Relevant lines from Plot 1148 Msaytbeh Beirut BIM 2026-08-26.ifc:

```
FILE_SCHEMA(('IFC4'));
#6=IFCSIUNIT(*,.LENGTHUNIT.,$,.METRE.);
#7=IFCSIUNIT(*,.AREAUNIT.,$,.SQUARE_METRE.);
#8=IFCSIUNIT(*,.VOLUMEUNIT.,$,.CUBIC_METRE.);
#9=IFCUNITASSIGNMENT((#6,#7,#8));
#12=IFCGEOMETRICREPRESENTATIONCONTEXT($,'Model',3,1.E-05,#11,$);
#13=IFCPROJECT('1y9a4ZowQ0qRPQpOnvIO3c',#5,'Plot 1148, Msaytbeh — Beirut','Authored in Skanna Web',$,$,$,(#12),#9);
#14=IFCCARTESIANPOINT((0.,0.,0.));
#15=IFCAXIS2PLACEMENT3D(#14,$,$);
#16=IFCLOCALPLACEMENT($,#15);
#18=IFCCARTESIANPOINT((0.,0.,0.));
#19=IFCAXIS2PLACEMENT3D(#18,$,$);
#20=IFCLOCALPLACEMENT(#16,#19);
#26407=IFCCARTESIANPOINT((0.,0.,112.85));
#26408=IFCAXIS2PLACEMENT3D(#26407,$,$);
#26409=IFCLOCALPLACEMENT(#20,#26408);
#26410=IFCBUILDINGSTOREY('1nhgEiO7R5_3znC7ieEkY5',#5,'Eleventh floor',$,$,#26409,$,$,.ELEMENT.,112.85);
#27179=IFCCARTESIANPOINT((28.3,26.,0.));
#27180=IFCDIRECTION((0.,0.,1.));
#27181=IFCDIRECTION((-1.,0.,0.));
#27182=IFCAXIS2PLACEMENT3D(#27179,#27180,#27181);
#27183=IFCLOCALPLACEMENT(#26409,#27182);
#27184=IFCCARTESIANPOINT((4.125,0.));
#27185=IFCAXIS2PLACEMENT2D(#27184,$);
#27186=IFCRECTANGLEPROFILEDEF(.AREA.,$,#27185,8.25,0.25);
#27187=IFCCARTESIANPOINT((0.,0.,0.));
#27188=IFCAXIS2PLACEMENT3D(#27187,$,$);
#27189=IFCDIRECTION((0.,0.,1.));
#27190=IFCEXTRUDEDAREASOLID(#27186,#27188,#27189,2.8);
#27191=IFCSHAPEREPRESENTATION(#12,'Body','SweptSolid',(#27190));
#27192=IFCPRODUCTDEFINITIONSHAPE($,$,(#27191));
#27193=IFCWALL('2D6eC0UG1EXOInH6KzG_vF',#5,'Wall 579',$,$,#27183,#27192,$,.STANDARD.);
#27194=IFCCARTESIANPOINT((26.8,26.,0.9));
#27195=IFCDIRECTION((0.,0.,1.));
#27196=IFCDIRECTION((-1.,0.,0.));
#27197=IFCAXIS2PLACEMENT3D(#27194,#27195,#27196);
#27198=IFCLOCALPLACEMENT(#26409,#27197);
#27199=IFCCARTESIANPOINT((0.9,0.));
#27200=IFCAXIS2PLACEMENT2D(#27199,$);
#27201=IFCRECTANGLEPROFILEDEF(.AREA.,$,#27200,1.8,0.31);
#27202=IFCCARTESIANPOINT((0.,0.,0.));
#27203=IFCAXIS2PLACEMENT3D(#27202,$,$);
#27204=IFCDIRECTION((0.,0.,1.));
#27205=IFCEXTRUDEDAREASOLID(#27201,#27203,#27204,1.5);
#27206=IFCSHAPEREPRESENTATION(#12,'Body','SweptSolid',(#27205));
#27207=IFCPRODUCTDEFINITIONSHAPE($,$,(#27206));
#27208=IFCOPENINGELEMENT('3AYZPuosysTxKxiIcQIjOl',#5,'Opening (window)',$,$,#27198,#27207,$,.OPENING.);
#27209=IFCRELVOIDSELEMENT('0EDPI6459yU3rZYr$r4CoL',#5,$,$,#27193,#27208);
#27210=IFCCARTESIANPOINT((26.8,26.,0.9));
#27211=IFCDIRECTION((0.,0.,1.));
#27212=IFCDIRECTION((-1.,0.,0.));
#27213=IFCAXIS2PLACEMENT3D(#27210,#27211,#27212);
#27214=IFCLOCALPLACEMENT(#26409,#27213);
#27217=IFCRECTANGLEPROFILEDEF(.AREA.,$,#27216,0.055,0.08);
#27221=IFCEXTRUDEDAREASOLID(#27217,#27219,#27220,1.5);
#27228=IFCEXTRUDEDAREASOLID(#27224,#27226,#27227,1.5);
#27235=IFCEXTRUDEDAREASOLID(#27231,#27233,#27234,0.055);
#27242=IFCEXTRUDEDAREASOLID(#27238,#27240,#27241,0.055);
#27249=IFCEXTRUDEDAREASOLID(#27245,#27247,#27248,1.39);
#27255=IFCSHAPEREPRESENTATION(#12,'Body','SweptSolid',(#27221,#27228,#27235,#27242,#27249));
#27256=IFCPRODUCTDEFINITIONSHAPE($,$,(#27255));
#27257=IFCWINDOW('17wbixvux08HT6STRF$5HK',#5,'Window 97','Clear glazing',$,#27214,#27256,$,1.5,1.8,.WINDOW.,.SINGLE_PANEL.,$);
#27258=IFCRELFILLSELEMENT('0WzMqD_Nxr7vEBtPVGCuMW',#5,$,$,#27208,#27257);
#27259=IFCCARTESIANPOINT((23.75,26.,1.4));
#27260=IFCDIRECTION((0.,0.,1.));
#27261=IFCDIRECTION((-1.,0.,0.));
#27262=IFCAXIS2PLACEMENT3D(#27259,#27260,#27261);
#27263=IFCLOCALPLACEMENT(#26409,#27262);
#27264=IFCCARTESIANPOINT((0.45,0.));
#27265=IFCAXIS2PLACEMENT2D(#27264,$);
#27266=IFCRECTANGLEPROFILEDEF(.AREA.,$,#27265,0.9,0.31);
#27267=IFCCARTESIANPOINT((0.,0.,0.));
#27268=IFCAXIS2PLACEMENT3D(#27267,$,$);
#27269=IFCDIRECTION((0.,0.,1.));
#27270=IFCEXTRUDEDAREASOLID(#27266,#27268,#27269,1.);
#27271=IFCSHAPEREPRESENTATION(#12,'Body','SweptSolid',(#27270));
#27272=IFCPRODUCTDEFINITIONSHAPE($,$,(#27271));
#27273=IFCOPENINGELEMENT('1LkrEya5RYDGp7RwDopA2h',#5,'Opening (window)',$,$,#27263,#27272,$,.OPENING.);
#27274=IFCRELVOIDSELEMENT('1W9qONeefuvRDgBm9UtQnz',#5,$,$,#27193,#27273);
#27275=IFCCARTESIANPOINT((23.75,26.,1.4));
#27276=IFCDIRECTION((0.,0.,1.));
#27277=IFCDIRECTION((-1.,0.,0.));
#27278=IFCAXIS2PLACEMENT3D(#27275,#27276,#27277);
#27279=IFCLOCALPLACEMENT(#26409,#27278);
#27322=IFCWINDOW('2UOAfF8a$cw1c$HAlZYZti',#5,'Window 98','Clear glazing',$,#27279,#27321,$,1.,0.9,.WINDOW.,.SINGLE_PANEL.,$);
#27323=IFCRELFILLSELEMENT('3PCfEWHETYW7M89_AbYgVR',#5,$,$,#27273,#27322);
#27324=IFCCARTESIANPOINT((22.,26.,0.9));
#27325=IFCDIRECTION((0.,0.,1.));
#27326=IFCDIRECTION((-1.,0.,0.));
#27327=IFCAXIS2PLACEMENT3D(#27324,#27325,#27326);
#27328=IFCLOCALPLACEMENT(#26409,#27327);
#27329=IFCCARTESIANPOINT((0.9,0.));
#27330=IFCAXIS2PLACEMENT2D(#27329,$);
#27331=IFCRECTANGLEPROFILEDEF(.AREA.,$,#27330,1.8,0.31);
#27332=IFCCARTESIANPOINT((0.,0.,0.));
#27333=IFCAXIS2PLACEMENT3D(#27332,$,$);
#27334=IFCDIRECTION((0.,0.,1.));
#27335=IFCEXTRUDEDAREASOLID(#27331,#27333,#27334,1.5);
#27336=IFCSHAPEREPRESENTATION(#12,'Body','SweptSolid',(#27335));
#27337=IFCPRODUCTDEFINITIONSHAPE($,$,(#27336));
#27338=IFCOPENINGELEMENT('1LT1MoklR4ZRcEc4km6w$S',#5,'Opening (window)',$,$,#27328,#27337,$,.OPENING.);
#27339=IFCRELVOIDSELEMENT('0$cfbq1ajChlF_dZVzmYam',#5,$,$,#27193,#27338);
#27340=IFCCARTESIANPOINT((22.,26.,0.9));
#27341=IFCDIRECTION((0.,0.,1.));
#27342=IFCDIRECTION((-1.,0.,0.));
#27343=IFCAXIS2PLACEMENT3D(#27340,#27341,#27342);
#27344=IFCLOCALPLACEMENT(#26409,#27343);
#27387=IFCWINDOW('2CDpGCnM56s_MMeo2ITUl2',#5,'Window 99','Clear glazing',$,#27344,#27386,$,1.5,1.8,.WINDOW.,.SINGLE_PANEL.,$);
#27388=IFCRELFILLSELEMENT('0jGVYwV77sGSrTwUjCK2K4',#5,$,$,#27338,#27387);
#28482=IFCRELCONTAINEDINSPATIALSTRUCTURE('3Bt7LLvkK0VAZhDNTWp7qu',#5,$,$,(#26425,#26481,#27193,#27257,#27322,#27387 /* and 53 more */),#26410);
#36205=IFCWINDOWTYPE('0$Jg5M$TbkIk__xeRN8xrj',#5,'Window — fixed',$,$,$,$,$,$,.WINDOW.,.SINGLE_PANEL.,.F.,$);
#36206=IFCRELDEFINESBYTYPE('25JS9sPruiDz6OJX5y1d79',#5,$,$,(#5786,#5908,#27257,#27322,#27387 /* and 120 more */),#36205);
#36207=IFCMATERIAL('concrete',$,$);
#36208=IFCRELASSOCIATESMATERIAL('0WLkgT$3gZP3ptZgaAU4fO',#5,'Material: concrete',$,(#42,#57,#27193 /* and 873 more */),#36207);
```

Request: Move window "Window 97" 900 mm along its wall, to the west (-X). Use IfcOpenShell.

```python
import ifcopenshell
import ifcopenshell.api.geometry
import ifcopenshell.util.placement
import ifcopenshell.util.unit

model = ifcopenshell.open("Plot 1148 Msaytbeh Beirut BIM 2026-08-26.ifc")
unit_scale = ifcopenshell.util.unit.calculate_unit_scale(model)

window = model.by_guid("17wbixvux08HT6STRF$5HK")
opening = window.FillsVoids[0].RelatingOpeningElement
wall = opening.VoidsElements[0].RelatingBuildingElement

wall_matrix = ifcopenshell.util.placement.get_local_placement(wall.ObjectPlacement)
shift = wall_matrix[:3, 0] * 0.9 / unit_scale
before = ifcopenshell.util.placement.get_local_placement(window.ObjectPlacement)[:3, 3].copy()

# The window is not placed relative to its opening, so move both.
for product in (opening, window):
    matrix = ifcopenshell.util.placement.get_local_placement(product.ObjectPlacement)
    matrix[:3, 3] += shift
    ifcopenshell.api.geometry.edit_object_placement(model, product=product, matrix=matrix, is_si=False)

after = ifcopenshell.util.placement.get_local_placement(window.ObjectPlacement)[:3, 3]
print("window moved by", (after - before).round(3) + 0.0)

model.write("Plot 1148 Msaytbeh Beirut BIM 2026-08-26_v2.ifc")
```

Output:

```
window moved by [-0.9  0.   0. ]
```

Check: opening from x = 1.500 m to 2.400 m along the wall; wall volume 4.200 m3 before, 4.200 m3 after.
